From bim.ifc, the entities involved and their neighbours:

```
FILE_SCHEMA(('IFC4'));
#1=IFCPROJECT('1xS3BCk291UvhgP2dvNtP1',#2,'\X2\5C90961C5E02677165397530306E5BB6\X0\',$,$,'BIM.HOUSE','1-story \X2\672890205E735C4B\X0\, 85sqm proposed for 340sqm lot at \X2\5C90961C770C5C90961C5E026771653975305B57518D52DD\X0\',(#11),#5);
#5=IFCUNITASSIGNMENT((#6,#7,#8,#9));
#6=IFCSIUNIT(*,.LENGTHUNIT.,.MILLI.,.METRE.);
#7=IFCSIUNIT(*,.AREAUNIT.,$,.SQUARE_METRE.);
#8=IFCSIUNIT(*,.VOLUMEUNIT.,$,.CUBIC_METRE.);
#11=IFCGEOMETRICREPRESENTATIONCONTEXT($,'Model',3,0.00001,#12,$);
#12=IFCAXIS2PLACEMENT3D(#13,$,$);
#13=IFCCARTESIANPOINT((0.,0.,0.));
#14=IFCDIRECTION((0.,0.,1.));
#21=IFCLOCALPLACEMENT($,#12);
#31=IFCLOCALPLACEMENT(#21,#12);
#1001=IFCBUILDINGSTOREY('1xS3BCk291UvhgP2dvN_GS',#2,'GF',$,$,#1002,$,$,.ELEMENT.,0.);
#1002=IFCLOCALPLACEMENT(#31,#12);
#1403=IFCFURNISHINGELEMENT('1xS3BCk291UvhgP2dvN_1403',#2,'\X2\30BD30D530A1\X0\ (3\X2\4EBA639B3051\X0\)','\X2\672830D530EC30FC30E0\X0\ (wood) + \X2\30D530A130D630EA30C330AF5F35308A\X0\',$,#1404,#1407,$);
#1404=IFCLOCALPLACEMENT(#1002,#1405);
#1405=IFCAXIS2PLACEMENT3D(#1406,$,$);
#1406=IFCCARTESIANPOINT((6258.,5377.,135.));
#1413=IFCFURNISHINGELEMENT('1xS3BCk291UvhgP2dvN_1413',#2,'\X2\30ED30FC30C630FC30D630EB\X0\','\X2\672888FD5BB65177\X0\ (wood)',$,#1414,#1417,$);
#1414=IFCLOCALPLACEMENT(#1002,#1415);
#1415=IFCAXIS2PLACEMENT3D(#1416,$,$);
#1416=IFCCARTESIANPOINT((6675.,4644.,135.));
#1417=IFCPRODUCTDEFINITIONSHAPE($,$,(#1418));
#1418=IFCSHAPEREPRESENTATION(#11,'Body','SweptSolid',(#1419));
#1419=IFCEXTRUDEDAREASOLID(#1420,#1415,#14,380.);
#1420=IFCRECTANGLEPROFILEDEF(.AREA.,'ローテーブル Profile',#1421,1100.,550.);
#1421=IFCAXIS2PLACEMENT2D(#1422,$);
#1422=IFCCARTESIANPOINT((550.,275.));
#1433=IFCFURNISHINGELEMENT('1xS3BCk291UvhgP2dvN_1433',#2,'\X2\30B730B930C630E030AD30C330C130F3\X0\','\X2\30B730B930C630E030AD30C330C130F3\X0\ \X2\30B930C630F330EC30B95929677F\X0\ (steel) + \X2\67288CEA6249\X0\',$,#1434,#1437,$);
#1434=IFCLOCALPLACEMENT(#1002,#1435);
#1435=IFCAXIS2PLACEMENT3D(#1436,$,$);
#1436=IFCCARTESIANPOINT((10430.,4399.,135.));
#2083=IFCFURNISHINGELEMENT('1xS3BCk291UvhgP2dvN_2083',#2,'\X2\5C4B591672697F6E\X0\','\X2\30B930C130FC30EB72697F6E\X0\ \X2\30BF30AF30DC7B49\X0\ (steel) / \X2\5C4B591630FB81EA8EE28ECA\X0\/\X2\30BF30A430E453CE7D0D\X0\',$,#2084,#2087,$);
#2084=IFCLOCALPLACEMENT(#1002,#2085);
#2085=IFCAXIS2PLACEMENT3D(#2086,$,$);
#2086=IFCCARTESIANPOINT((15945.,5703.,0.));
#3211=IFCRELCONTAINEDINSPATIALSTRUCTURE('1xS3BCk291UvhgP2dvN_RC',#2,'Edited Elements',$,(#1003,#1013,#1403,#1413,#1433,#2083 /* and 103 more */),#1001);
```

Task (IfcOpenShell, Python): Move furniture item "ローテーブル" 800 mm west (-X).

```python
import ifcopenshell
import ifcopenshell.api.geometry
import ifcopenshell.util.placement

model = ifcopenshell.open("bim.ifc")

item = model.by_guid("1xS3BCk291UvhgP2dvN_1413")
matrix = ifcopenshell.util.placement.get_local_placement(item.ObjectPlacement)
matrix[0, 3] -= 800.0
ifcopenshell.api.geometry.edit_object_placement(model, product=item, matrix=matrix, is_si=False)

print(ifcopenshell.util.placement.get_local_placement(item.ObjectPlacement).round(3) + 0.0)

model.write("bim_v2.ifc")
```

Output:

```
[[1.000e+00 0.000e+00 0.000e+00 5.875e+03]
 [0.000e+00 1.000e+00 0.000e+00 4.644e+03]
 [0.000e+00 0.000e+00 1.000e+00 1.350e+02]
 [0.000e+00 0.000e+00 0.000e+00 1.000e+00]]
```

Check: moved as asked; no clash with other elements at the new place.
